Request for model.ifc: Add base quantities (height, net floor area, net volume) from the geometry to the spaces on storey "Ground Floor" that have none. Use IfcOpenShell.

First a look at what the model holds.

```python
import ifcopenshell
import ifcopenshell.util.element
import ifcopenshell.util.unit

model = ifcopenshell.open("model.ifc")
print(model.schema)
for unit_type in ("LENGTHUNIT", "AREAUNIT", "VOLUMEUNIT"):
    print(unit_type, ifcopenshell.util.unit.calculate_unit_scale(model, unit_type))
storey = next(s for s in model.by_type("IfcBuildingStorey") if s.Name == "Ground Floor")
spaces = [e for e in ifcopenshell.util.element.get_decomposition(storey) if e.is_a("IfcSpace")]
for e in sorted(spaces, key=lambda e: e.id()):
    print(e.id(), e.is_a(), e.Name, list(ifcopenshell.util.element.get_psets(e, qtos_only=True)), sep=" | ")
```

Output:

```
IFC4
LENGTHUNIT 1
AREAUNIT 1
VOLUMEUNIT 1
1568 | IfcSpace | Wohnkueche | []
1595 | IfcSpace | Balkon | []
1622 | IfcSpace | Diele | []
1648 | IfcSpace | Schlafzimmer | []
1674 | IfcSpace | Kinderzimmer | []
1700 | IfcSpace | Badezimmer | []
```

```python
import ifcopenshell
import ifcopenshell.api.pset
import ifcopenshell.geom
import ifcopenshell.util.element
import ifcopenshell.util.shape
import ifcopenshell.util.unit

model = ifcopenshell.open("model.ifc")
unit_scale = ifcopenshell.util.unit.calculate_unit_scale(model)
area_scale = ifcopenshell.util.unit.calculate_unit_scale(model, "AREAUNIT")
volume_scale = ifcopenshell.util.unit.calculate_unit_scale(model, "VOLUMEUNIT")
settings = ifcopenshell.geom.settings()

storey = next(s for s in model.by_type("IfcBuildingStorey") if s.Name == "Ground Floor")
spaces = [e for e in ifcopenshell.util.element.get_decomposition(storey) if e.is_a("IfcSpace")]

for e in sorted(spaces, key=lambda e: e.id()):
    if ifcopenshell.util.element.get_psets(e, qtos_only=True, should_inherit=False):
        continue
    # Geometry comes back in metres, in the element's own axes.
    shape = ifcopenshell.geom.create_shape(settings, e)
    values = {
        "Height": ifcopenshell.util.shape.get_z(shape.geometry) / unit_scale,
        "NetFloorArea": ifcopenshell.util.shape.get_footprint_area(shape.geometry) / area_scale,
        "NetVolume": ifcopenshell.util.shape.get_volume(shape.geometry) / volume_scale,
    }
    qto = ifcopenshell.api.pset.add_qto(model, product=e, name="Qto_SpaceBaseQuantities")
    ifcopenshell.api.pset.edit_qto(model, qto=qto, properties=values)
    print(e.id(), {k: round(v, 3) for k, v in values.items()})

model.write("model_rev.ifc")
```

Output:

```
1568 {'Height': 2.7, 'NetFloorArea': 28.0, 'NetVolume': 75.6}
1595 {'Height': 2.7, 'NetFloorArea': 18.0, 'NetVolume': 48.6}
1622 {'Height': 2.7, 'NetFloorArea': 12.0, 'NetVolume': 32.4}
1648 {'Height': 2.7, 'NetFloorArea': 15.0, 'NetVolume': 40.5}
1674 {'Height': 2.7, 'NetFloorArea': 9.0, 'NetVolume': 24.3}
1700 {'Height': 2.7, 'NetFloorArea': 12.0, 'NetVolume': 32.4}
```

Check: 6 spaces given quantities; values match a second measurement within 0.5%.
